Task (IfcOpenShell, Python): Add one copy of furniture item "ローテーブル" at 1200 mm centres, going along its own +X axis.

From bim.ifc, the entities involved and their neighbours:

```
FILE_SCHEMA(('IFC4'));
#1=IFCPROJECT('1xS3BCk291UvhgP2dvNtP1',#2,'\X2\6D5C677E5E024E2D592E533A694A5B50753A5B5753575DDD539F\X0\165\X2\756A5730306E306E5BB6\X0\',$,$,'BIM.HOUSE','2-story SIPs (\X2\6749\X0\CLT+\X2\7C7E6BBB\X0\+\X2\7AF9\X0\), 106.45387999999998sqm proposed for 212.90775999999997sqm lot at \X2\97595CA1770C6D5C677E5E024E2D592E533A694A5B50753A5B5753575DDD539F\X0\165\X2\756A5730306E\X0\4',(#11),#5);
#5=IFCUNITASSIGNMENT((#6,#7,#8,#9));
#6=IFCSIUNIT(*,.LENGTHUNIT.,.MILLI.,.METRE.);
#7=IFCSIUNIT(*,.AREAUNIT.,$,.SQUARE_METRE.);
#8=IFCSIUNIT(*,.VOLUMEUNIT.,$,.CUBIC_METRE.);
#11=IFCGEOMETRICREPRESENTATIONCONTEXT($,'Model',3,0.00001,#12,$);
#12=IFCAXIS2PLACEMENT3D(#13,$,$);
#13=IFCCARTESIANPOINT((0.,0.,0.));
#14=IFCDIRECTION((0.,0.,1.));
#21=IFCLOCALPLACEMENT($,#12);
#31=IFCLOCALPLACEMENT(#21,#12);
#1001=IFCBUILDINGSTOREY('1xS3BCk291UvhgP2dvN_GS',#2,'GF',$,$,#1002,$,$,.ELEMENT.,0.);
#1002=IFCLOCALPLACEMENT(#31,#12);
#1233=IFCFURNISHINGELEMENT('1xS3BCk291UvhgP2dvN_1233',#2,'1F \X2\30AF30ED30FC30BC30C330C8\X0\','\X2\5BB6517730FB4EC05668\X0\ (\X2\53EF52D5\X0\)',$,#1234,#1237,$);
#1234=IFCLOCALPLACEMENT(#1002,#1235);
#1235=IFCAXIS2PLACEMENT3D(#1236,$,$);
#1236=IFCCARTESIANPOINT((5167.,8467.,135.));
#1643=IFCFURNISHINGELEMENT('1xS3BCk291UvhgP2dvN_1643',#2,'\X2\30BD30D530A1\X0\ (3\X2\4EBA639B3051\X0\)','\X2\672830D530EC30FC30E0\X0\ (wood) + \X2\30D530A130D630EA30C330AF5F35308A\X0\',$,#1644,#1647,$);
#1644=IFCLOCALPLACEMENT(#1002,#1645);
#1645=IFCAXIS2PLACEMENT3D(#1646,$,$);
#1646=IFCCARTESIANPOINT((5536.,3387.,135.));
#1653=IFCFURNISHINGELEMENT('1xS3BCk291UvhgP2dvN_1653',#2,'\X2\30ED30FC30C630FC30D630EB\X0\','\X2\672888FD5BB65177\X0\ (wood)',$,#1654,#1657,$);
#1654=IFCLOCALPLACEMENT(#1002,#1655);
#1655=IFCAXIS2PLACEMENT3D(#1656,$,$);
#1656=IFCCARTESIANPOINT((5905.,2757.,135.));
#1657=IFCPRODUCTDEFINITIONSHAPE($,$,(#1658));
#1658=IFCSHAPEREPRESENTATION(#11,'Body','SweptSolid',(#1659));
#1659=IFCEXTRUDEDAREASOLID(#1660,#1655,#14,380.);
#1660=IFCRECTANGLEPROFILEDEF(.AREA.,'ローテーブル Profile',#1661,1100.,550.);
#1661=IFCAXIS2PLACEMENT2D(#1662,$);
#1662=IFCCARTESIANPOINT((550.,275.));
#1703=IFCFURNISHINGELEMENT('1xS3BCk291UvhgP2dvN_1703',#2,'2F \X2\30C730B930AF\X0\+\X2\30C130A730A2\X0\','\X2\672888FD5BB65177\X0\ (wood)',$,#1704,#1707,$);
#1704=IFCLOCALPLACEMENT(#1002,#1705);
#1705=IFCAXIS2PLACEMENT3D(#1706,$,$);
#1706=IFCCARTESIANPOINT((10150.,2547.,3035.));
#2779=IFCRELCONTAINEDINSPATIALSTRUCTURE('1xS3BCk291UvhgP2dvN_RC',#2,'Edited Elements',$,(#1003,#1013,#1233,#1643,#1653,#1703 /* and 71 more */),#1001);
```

```python
import ifcopenshell
import ifcopenshell.api.geometry
import ifcopenshell.api.root
import ifcopenshell.util.element
import ifcopenshell.util.placement
import ifcopenshell.util.unit

model = ifcopenshell.open("bim.ifc")
unit_scale = ifcopenshell.util.unit.calculate_unit_scale(model)


def reuse_history(source, copy):
    """copy_class also copies each property set's owner history, people and application; keep the originals."""
    for rel in copy.IsDefinedBy:
        if rel.is_a("IfcRelDefinesByProperties") and (history := rel.RelatingPropertyDefinition.OwnerHistory):
            rel.RelatingPropertyDefinition.OwnerHistory = source.OwnerHistory
            ifcopenshell.util.element.remove_deep2(model, history)


source = model.by_guid("1xS3BCk291UvhgP2dvN_1653")
base = ifcopenshell.util.placement.get_local_placement(source.ObjectPlacement)
step = base[:3, 0] * 1.2 / unit_scale

for i in range(1, 2):
    copy = ifcopenshell.api.root.copy_class(model, product=source)
    copy.Representation = ifcopenshell.util.element.copy_deep(
        model, source.Representation, exclude=["IfcGeometricRepresentationContext", "IfcRepresentationMap"]
    )
    reuse_history(source, copy)
    matrix = base.copy()
    matrix[:3, 3] += i * step
    print("added at", matrix[:3, 3].round(3) + 0.0)
    ifcopenshell.api.geometry.edit_object_placement(model, product=copy, matrix=matrix, is_si=False)

model.write("bim_updated.ifc")
```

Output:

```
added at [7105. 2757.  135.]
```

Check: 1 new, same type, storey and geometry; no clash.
